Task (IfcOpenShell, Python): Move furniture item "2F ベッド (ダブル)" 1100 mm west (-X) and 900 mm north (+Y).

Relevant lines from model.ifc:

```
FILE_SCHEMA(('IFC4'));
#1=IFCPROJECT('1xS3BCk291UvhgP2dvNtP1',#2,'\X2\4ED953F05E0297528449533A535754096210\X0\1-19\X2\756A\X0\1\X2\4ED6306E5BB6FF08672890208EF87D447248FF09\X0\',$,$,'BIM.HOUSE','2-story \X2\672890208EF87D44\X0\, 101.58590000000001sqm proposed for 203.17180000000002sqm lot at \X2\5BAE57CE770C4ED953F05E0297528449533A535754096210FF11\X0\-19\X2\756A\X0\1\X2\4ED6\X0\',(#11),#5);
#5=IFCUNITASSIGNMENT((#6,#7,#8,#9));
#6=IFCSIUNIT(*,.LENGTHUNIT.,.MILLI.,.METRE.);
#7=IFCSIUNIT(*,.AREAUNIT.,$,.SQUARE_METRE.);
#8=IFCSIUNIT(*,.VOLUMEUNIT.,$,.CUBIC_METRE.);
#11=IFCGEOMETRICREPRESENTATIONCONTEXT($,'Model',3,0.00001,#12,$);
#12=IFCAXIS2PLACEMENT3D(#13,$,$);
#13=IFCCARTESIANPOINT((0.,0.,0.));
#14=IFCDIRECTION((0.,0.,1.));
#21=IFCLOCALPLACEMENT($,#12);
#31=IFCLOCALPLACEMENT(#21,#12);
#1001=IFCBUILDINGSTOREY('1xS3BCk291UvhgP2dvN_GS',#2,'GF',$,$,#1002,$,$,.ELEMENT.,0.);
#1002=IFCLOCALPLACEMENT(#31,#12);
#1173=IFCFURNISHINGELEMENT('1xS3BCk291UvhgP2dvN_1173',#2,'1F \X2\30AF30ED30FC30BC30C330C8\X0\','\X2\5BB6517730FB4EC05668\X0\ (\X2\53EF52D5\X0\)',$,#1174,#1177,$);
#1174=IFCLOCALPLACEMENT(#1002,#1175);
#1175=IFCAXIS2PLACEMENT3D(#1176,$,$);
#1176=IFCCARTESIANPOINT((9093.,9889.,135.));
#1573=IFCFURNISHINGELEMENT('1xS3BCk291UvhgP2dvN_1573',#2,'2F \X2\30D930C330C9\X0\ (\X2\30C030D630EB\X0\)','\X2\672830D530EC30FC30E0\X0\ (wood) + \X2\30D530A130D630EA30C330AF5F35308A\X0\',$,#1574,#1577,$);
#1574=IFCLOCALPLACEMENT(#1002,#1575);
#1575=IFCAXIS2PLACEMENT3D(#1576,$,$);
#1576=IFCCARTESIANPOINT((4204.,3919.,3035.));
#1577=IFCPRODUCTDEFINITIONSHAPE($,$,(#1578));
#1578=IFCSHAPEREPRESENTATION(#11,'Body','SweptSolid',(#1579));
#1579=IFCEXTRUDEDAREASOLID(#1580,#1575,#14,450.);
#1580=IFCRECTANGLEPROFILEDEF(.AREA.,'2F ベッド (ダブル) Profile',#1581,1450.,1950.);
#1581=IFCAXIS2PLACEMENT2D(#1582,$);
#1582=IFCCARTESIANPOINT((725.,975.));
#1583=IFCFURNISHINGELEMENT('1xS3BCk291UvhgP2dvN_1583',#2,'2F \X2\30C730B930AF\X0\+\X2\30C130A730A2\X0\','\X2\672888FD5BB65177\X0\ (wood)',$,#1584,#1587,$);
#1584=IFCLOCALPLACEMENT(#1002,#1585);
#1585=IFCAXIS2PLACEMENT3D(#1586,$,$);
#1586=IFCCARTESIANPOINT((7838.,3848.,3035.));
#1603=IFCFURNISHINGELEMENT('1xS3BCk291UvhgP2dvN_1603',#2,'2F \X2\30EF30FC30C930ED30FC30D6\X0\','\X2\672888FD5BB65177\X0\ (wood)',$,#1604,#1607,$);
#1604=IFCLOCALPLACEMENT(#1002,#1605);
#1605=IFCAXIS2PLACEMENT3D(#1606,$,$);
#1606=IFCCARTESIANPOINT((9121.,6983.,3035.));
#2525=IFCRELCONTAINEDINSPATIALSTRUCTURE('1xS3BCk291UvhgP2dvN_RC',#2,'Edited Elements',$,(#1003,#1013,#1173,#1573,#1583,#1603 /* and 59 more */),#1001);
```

```python
import ifcopenshell
import ifcopenshell.api.geometry
import ifcopenshell.util.placement
import ifcopenshell.util.unit

model = ifcopenshell.open("model.ifc")
unit_scale = ifcopenshell.util.unit.calculate_unit_scale(model)

item = model.by_guid("1xS3BCk291UvhgP2dvN_1573")
matrix = ifcopenshell.util.placement.get_local_placement(item.ObjectPlacement)
matrix[0, 3] -= 1.1 / unit_scale
matrix[1, 3] += 0.9 / unit_scale
ifcopenshell.api.geometry.edit_object_placement(model, product=item, matrix=matrix, is_si=False)

print(ifcopenshell.util.placement.get_local_placement(item.ObjectPlacement).round(3) + 0.0)

model.write("model_updated.ifc")
```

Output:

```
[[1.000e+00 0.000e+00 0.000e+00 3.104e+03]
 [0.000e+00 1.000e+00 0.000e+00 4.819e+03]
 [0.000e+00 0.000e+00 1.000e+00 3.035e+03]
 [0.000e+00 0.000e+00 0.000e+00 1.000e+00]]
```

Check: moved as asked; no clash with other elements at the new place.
